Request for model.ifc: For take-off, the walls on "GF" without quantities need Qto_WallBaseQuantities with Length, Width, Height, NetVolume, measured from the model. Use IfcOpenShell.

First a look at what the model holds.

```python
import ifcopenshell
import ifcopenshell.util.element
import ifcopenshell.util.unit

model = ifcopenshell.open("model.ifc")
print(model.schema)
for unit_type in ("LENGTHUNIT", "AREAUNIT", "VOLUMEUNIT"):
    print(unit_type, ifcopenshell.util.unit.calculate_unit_scale(model, unit_type))
storey = next(s for s in model.by_type("IfcBuildingStorey") if s.Name == "GF")
walls = [e for e in ifcopenshell.util.element.get_decomposition(storey) if e.is_a("IfcWall")]
for e in sorted(walls, key=lambda e: e.id()):
    print(e.id(), e.is_a(), e.Name, list(ifcopenshell.util.element.get_psets(e, qtos_only=True)), sep=" | ")
```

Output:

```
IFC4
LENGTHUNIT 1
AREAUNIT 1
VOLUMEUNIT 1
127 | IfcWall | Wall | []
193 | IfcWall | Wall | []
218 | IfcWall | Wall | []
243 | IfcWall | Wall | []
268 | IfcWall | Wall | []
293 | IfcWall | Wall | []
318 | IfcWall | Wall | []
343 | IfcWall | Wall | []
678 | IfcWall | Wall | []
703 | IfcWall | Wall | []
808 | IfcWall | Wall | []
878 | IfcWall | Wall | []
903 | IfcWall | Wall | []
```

```python
import ifcopenshell
import ifcopenshell.api.pset
import ifcopenshell.geom
import ifcopenshell.util.element
import ifcopenshell.util.shape
import ifcopenshell.util.unit

model = ifcopenshell.open("model.ifc")
unit_scale = ifcopenshell.util.unit.calculate_unit_scale(model)
volume_scale = ifcopenshell.util.unit.calculate_unit_scale(model, "VOLUMEUNIT")
settings = ifcopenshell.geom.settings()

storey = next(s for s in model.by_type("IfcBuildingStorey") if s.Name == "GF")
walls = [e for e in ifcopenshell.util.element.get_decomposition(storey) if e.is_a("IfcWall")]

for e in sorted(walls, key=lambda e: e.id()):
    if ifcopenshell.util.element.get_psets(e, qtos_only=True, should_inherit=False):
        continue
    # Geometry comes back in metres, in the element's own axes.
    shape = ifcopenshell.geom.create_shape(settings, e)
    values = {
        "Length": ifcopenshell.util.shape.get_x(shape.geometry) / unit_scale,
        "Width": ifcopenshell.util.shape.get_y(shape.geometry) / unit_scale,
        "Height": ifcopenshell.util.shape.get_z(shape.geometry) / unit_scale,
        "NetVolume": ifcopenshell.util.shape.get_volume(shape.geometry) / volume_scale,
    }
    qto = ifcopenshell.api.pset.add_qto(model, product=e, name="Qto_WallBaseQuantities")
    ifcopenshell.api.pset.edit_qto(model, qto=qto, properties=values)
    print(e.id(), {k: round(v, 3) for k, v in values.items()})

model.write("model_updated.ifc")
```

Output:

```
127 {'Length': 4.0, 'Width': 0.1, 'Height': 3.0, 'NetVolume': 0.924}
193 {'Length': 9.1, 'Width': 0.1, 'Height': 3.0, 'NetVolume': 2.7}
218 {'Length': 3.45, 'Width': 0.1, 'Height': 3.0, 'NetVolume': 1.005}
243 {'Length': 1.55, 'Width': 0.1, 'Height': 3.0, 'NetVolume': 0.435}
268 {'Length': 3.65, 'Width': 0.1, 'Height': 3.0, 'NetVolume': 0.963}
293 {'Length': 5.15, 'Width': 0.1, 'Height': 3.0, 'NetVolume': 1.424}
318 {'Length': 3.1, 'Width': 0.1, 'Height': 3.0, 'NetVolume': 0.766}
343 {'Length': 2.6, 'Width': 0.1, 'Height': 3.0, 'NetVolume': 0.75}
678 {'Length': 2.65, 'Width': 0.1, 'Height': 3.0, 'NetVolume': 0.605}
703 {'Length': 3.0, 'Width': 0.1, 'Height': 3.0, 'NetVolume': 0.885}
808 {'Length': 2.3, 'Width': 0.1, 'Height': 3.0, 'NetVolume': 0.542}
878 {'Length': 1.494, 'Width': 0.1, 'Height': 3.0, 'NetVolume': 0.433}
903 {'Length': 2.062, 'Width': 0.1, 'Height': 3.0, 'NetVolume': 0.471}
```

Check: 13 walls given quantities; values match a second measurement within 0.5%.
